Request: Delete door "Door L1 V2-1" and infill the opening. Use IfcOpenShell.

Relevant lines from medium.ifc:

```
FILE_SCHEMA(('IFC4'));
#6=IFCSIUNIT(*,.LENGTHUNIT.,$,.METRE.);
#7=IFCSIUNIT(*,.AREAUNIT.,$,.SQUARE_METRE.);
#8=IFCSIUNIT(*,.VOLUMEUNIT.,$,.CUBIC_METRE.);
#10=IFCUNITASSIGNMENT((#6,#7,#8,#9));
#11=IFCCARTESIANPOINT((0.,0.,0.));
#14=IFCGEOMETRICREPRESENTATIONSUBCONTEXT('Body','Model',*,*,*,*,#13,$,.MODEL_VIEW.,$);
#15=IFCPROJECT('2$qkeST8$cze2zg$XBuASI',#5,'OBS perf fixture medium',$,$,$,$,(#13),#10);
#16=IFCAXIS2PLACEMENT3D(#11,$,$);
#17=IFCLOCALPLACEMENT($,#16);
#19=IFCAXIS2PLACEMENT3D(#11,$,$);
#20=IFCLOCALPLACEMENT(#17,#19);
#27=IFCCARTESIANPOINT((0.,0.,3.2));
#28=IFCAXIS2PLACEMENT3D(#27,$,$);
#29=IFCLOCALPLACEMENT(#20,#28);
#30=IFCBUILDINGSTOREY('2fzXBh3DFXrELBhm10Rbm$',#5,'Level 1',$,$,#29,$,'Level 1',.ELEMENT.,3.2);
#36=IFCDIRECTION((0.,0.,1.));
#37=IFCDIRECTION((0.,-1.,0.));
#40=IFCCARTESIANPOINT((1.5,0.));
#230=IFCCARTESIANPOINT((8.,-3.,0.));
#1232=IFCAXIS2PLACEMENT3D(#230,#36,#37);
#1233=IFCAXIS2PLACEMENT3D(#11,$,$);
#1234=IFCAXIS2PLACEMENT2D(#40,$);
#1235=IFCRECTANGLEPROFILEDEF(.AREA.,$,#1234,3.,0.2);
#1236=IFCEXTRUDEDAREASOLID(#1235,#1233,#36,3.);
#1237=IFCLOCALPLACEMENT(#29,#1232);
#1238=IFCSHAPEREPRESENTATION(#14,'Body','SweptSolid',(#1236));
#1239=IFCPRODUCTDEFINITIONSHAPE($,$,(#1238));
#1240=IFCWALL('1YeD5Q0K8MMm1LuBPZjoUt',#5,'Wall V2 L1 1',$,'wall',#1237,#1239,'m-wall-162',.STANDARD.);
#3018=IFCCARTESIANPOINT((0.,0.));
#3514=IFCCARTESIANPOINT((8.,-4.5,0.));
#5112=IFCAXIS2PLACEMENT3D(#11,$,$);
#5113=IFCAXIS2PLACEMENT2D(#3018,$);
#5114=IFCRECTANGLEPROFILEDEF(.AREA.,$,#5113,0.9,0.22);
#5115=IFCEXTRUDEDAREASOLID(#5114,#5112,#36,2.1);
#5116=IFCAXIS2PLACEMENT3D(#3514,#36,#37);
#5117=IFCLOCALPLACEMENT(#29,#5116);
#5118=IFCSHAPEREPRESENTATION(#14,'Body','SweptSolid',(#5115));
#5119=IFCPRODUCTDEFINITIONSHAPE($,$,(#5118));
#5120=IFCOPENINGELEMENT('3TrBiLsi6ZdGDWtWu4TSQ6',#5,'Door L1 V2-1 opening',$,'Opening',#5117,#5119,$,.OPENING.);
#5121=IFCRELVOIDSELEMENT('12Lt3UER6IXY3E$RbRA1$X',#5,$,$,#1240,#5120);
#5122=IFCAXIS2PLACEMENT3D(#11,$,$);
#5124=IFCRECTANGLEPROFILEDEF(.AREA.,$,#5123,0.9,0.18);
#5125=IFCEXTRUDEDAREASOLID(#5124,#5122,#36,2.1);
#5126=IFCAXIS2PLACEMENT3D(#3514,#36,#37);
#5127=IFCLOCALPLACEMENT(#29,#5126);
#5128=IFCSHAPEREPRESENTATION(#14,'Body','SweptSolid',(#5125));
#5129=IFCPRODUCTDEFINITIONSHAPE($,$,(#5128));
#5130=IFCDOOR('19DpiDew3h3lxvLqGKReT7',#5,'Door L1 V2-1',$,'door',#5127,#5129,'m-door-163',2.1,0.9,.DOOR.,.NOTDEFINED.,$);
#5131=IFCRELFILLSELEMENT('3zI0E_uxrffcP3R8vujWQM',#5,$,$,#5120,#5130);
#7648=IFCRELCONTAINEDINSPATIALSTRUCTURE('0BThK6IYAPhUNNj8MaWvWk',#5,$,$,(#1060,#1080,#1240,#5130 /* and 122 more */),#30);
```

```python
import ifcopenshell
import ifcopenshell.api.feature
import ifcopenshell.api.root
import ifcopenshell.geom
import ifcopenshell.util.shape

model = ifcopenshell.open("medium.ifc")
settings = ifcopenshell.geom.settings()


def volume(element):
    """Net volume in cubic metres, openings subtracted."""
    shape = ifcopenshell.geom.create_shape(settings, element)
    return ifcopenshell.util.shape.get_volume(shape.geometry)


door = model.by_guid("19DpiDew3h3lxvLqGKReT7")
opening = door.FillsVoids[0].RelatingOpeningElement
wall = opening.VoidsElements[0].RelatingBuildingElement
before = volume(wall)

ifcopenshell.api.root.remove_product(model, product=door)
ifcopenshell.api.feature.remove_feature(model, feature=opening)

after = volume(wall)

print(f"wall volume {before:.3f} -> {after:.3f} m3")

model.write("medium_v2.ifc")
```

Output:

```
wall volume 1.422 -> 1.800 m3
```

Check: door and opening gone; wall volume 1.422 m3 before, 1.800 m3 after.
